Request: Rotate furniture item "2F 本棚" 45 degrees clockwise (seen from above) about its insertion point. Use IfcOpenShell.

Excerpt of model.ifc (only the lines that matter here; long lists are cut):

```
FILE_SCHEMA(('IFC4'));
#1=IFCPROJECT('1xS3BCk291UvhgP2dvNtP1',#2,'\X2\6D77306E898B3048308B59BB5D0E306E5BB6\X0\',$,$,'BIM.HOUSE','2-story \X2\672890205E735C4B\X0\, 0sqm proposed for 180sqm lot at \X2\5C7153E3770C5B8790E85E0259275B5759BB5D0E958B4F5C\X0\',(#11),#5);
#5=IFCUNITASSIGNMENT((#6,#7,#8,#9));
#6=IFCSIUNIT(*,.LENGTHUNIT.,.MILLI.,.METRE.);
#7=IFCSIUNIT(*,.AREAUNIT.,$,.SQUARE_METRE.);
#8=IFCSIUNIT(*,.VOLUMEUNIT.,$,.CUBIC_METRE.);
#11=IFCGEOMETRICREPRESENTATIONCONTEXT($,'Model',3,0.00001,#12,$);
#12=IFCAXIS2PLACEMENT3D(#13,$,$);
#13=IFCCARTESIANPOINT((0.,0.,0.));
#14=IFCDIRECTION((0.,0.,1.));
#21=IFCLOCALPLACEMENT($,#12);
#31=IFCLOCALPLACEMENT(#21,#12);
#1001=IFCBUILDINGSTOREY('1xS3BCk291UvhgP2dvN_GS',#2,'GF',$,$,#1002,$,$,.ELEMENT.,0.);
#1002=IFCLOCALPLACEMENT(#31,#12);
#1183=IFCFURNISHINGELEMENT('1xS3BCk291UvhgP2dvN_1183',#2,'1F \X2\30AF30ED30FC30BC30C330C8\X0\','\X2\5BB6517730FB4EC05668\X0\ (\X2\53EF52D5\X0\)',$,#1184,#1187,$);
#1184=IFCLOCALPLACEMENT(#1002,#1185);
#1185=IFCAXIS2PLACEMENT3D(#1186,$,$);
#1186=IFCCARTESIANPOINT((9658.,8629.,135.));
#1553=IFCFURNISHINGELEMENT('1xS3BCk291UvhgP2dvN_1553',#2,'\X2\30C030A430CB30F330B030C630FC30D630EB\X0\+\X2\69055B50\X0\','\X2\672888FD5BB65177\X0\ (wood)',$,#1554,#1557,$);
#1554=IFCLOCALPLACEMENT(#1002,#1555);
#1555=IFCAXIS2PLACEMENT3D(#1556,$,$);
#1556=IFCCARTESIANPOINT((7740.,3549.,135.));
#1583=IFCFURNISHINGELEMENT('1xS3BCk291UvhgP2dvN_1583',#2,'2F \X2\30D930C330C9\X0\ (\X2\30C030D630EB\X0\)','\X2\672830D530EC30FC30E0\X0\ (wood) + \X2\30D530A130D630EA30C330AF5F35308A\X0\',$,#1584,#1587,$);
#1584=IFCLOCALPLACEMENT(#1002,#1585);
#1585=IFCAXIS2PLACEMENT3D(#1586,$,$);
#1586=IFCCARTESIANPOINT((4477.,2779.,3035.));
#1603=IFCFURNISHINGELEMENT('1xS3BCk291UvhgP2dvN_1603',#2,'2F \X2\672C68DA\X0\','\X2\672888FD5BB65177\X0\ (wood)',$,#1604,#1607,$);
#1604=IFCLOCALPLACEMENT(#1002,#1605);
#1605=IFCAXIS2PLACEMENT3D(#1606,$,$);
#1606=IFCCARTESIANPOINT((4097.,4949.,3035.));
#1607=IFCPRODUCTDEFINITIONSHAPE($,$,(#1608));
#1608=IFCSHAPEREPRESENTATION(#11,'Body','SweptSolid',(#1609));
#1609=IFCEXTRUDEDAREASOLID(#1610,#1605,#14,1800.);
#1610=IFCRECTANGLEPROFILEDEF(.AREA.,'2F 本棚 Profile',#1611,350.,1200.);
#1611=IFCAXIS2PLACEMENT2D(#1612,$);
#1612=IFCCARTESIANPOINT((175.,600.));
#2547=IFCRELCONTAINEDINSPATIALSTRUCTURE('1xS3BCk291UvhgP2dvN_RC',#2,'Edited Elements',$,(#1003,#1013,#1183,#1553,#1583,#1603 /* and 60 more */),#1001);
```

```python
import ifcopenshell
import ifcopenshell.api.geometry
import ifcopenshell.util.placement

model = ifcopenshell.open("model.ifc")

item = model.by_guid("1xS3BCk291UvhgP2dvN_1603")
matrix = ifcopenshell.util.placement.get_local_placement(item.ObjectPlacement)
matrix = matrix @ ifcopenshell.util.placement.rotation(-45, "Z")
ifcopenshell.api.geometry.edit_object_placement(model, product=item, matrix=matrix, is_si=False)

print(ifcopenshell.util.placement.get_local_placement(item.ObjectPlacement).round(3) + 0.0)

model.write("model_rev.ifc")
```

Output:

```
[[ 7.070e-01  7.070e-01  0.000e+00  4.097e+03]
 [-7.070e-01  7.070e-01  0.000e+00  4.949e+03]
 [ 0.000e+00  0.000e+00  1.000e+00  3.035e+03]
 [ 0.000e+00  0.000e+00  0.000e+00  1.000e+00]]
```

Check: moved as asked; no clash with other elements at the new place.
